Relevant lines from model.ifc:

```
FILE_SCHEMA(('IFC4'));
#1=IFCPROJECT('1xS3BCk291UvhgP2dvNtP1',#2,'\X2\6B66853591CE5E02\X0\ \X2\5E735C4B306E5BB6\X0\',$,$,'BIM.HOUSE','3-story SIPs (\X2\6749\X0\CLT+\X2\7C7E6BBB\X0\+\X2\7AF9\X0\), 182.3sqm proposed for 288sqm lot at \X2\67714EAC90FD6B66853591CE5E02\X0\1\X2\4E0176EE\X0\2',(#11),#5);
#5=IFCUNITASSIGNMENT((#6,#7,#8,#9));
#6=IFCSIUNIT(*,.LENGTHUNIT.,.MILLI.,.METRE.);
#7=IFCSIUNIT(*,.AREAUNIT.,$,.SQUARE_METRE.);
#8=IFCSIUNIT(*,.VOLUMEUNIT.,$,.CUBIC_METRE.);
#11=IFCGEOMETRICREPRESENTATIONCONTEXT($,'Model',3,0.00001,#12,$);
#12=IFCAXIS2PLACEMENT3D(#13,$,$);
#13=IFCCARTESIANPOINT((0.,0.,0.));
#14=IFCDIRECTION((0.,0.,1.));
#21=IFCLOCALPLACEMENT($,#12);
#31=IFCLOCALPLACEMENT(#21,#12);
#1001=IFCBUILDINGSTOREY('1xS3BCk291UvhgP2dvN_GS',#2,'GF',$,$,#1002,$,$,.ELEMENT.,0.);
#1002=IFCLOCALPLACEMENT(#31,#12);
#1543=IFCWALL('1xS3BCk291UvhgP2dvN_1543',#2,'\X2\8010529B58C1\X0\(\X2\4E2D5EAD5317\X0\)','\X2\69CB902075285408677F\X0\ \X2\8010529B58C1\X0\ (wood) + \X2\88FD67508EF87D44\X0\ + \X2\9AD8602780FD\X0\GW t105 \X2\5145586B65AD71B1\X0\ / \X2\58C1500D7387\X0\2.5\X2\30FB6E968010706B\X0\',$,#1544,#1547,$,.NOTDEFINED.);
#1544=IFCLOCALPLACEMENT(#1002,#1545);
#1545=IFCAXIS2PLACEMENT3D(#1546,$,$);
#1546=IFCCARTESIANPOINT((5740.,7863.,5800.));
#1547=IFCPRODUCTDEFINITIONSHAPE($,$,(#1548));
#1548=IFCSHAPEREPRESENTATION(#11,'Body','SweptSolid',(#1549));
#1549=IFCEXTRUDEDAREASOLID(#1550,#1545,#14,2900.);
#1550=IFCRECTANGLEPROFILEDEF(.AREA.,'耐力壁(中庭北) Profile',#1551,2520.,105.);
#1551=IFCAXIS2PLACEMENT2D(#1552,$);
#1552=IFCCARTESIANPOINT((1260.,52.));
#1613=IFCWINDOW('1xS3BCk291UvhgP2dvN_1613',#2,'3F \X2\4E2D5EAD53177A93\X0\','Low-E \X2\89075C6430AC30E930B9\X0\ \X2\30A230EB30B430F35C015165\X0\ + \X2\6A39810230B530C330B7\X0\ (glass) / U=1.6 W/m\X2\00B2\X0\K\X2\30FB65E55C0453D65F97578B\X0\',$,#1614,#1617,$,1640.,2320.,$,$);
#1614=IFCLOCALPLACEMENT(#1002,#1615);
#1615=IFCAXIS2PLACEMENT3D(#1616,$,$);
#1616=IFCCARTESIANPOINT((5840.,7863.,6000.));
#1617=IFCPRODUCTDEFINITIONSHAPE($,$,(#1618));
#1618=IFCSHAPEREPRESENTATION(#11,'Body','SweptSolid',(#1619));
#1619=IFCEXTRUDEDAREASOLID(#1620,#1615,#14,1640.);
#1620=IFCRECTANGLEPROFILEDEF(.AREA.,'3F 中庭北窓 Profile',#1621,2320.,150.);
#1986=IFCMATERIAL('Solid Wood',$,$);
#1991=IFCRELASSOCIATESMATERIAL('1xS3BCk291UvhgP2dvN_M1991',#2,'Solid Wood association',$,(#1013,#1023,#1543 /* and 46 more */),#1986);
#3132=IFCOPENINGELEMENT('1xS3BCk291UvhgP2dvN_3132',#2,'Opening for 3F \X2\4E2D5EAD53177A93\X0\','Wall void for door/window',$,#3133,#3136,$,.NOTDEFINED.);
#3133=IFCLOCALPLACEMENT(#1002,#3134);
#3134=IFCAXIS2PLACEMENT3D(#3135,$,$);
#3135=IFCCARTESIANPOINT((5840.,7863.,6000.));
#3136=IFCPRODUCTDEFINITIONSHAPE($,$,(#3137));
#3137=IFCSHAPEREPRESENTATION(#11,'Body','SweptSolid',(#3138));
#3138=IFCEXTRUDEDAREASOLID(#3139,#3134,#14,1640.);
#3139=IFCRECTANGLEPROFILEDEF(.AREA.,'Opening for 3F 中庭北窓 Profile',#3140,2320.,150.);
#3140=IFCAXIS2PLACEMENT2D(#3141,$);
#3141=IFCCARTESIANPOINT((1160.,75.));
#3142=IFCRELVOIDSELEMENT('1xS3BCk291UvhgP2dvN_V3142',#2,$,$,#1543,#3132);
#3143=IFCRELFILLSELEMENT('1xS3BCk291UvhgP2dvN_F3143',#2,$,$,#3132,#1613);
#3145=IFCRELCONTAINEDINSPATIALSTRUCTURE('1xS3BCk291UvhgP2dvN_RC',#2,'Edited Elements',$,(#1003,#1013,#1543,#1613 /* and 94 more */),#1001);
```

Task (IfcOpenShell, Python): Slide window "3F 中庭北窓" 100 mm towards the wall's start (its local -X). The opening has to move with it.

```python
import ifcopenshell
import ifcopenshell.api.geometry
import ifcopenshell.util.placement

model = ifcopenshell.open("model.ifc")

window = model.by_guid("1xS3BCk291UvhgP2dvN_1613")
opening = window.FillsVoids[0].RelatingOpeningElement
wall = opening.VoidsElements[0].RelatingBuildingElement

wall_matrix = ifcopenshell.util.placement.get_local_placement(wall.ObjectPlacement)
shift = wall_matrix[:3, 0] * -100.0
before = ifcopenshell.util.placement.get_local_placement(window.ObjectPlacement)[:3, 3].copy()

# The window is not placed relative to its opening, so move both.
for product in (opening, window):
    matrix = ifcopenshell.util.placement.get_local_placement(product.ObjectPlacement)
    matrix[:3, 3] += shift
    ifcopenshell.api.geometry.edit_object_placement(model, product=product, matrix=matrix, is_si=False)

after = ifcopenshell.util.placement.get_local_placement(window.ObjectPlacement)[:3, 3]
print("window moved by", (after - before).round(3) + 0.0)

model.write("model_rev.ifc")
```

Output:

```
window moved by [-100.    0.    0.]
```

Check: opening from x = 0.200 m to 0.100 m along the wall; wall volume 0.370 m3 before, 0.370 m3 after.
